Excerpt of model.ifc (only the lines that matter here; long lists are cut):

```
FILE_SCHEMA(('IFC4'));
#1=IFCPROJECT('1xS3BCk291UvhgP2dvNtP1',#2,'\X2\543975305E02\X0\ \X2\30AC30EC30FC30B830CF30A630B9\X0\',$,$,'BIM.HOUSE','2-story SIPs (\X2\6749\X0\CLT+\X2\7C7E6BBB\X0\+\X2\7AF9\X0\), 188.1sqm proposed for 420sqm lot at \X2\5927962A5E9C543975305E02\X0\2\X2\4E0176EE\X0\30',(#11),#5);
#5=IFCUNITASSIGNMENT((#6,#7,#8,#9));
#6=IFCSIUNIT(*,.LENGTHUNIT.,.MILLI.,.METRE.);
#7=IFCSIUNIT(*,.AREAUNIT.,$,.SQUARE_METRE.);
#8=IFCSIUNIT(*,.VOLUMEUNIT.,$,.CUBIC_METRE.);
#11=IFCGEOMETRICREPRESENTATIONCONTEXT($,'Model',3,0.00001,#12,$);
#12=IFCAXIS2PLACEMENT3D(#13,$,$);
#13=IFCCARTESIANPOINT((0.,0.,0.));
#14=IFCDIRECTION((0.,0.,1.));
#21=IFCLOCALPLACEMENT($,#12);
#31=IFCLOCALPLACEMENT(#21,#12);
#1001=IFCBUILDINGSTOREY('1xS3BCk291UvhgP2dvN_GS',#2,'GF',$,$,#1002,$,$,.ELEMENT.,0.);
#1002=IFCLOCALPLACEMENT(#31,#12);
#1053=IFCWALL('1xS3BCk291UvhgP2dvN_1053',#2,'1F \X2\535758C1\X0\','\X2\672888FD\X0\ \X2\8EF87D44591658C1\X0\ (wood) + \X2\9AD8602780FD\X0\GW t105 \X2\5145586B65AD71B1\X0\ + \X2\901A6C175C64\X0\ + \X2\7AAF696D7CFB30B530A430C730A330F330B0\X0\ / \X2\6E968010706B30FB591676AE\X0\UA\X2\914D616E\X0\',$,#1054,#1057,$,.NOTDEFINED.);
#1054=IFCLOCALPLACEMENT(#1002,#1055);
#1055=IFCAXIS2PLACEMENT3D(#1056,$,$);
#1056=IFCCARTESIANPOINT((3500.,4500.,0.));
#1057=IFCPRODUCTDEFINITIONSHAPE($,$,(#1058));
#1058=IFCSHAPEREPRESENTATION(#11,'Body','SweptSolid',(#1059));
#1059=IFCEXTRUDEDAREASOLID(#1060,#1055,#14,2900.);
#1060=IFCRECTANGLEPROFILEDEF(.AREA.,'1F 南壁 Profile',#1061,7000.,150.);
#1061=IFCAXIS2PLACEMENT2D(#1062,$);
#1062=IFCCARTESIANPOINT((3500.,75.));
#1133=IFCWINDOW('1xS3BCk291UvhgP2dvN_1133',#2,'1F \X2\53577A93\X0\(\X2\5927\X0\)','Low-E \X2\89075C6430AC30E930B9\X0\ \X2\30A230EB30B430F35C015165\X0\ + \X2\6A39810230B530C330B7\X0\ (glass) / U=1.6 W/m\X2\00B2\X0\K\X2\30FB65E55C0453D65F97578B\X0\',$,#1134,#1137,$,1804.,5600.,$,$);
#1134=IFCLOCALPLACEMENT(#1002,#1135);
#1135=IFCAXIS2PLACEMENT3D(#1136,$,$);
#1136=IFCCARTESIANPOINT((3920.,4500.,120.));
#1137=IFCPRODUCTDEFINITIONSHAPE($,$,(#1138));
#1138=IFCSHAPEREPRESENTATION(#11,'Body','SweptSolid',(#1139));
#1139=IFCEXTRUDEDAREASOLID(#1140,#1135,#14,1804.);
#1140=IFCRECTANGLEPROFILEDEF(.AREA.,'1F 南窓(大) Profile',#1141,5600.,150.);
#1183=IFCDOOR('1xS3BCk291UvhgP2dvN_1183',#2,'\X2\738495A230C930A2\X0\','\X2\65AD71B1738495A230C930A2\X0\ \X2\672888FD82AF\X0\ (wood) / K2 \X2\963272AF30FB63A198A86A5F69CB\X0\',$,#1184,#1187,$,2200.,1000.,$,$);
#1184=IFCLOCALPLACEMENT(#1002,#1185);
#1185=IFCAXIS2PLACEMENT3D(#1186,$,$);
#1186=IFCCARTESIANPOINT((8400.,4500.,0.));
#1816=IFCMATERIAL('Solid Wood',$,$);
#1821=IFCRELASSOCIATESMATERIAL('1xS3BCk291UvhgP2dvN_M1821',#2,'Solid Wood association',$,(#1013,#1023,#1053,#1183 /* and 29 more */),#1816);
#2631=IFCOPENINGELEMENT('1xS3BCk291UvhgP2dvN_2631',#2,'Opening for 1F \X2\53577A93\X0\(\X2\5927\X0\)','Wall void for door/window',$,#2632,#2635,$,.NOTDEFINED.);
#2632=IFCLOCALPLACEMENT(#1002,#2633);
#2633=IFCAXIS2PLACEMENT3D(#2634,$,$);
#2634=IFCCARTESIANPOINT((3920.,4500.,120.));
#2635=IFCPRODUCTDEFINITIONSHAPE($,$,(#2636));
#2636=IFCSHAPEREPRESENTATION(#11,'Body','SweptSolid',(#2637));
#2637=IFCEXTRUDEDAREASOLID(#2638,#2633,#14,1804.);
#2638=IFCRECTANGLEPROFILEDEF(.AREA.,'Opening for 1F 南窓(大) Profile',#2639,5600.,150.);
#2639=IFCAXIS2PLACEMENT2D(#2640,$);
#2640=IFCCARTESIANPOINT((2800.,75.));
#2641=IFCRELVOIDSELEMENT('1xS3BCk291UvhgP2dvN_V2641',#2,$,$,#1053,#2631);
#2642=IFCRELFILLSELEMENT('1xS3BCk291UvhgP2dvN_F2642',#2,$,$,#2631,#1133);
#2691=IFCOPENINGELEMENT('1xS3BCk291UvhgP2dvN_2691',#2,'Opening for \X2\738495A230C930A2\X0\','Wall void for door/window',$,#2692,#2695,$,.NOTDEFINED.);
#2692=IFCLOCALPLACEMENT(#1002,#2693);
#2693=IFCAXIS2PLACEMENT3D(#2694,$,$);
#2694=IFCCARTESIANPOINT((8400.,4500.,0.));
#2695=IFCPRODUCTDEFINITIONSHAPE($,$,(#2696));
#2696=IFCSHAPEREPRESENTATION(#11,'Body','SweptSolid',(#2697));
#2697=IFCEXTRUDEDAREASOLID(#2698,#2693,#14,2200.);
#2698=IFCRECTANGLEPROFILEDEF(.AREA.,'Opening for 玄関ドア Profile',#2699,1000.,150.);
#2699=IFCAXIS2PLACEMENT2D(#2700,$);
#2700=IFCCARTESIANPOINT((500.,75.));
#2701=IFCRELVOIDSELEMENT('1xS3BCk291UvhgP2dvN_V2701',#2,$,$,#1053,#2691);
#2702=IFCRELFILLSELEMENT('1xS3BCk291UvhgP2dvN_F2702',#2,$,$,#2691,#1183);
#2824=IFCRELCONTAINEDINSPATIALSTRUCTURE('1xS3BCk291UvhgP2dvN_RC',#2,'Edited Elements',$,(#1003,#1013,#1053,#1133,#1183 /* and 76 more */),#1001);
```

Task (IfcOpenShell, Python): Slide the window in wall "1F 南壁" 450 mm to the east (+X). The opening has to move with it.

```python
import ifcopenshell
import ifcopenshell.api.geometry
import ifcopenshell.util.placement
import ifcopenshell.util.unit

model = ifcopenshell.open("model.ifc")
unit_scale = ifcopenshell.util.unit.calculate_unit_scale(model)

window = model.by_guid("1xS3BCk291UvhgP2dvN_1133")
opening = window.FillsVoids[0].RelatingOpeningElement
wall = opening.VoidsElements[0].RelatingBuildingElement

wall_matrix = ifcopenshell.util.placement.get_local_placement(wall.ObjectPlacement)
shift = wall_matrix[:3, 0] * 0.45 / unit_scale
before = ifcopenshell.util.placement.get_local_placement(window.ObjectPlacement)[:3, 3].copy()

# The window is not placed relative to its opening, so move both.
for product in (opening, window):
    matrix = ifcopenshell.util.placement.get_local_placement(product.ObjectPlacement)
    matrix[:3, 3] += shift
    ifcopenshell.api.geometry.edit_object_placement(model, product=product, matrix=matrix, is_si=False)

after = ifcopenshell.util.placement.get_local_placement(window.ObjectPlacement)[:3, 3]
print("window moved by", (after - before).round(3) + 0.0)

model.write("model_v2.ifc")
```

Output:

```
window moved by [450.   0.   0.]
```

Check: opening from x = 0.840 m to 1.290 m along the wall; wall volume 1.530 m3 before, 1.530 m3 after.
